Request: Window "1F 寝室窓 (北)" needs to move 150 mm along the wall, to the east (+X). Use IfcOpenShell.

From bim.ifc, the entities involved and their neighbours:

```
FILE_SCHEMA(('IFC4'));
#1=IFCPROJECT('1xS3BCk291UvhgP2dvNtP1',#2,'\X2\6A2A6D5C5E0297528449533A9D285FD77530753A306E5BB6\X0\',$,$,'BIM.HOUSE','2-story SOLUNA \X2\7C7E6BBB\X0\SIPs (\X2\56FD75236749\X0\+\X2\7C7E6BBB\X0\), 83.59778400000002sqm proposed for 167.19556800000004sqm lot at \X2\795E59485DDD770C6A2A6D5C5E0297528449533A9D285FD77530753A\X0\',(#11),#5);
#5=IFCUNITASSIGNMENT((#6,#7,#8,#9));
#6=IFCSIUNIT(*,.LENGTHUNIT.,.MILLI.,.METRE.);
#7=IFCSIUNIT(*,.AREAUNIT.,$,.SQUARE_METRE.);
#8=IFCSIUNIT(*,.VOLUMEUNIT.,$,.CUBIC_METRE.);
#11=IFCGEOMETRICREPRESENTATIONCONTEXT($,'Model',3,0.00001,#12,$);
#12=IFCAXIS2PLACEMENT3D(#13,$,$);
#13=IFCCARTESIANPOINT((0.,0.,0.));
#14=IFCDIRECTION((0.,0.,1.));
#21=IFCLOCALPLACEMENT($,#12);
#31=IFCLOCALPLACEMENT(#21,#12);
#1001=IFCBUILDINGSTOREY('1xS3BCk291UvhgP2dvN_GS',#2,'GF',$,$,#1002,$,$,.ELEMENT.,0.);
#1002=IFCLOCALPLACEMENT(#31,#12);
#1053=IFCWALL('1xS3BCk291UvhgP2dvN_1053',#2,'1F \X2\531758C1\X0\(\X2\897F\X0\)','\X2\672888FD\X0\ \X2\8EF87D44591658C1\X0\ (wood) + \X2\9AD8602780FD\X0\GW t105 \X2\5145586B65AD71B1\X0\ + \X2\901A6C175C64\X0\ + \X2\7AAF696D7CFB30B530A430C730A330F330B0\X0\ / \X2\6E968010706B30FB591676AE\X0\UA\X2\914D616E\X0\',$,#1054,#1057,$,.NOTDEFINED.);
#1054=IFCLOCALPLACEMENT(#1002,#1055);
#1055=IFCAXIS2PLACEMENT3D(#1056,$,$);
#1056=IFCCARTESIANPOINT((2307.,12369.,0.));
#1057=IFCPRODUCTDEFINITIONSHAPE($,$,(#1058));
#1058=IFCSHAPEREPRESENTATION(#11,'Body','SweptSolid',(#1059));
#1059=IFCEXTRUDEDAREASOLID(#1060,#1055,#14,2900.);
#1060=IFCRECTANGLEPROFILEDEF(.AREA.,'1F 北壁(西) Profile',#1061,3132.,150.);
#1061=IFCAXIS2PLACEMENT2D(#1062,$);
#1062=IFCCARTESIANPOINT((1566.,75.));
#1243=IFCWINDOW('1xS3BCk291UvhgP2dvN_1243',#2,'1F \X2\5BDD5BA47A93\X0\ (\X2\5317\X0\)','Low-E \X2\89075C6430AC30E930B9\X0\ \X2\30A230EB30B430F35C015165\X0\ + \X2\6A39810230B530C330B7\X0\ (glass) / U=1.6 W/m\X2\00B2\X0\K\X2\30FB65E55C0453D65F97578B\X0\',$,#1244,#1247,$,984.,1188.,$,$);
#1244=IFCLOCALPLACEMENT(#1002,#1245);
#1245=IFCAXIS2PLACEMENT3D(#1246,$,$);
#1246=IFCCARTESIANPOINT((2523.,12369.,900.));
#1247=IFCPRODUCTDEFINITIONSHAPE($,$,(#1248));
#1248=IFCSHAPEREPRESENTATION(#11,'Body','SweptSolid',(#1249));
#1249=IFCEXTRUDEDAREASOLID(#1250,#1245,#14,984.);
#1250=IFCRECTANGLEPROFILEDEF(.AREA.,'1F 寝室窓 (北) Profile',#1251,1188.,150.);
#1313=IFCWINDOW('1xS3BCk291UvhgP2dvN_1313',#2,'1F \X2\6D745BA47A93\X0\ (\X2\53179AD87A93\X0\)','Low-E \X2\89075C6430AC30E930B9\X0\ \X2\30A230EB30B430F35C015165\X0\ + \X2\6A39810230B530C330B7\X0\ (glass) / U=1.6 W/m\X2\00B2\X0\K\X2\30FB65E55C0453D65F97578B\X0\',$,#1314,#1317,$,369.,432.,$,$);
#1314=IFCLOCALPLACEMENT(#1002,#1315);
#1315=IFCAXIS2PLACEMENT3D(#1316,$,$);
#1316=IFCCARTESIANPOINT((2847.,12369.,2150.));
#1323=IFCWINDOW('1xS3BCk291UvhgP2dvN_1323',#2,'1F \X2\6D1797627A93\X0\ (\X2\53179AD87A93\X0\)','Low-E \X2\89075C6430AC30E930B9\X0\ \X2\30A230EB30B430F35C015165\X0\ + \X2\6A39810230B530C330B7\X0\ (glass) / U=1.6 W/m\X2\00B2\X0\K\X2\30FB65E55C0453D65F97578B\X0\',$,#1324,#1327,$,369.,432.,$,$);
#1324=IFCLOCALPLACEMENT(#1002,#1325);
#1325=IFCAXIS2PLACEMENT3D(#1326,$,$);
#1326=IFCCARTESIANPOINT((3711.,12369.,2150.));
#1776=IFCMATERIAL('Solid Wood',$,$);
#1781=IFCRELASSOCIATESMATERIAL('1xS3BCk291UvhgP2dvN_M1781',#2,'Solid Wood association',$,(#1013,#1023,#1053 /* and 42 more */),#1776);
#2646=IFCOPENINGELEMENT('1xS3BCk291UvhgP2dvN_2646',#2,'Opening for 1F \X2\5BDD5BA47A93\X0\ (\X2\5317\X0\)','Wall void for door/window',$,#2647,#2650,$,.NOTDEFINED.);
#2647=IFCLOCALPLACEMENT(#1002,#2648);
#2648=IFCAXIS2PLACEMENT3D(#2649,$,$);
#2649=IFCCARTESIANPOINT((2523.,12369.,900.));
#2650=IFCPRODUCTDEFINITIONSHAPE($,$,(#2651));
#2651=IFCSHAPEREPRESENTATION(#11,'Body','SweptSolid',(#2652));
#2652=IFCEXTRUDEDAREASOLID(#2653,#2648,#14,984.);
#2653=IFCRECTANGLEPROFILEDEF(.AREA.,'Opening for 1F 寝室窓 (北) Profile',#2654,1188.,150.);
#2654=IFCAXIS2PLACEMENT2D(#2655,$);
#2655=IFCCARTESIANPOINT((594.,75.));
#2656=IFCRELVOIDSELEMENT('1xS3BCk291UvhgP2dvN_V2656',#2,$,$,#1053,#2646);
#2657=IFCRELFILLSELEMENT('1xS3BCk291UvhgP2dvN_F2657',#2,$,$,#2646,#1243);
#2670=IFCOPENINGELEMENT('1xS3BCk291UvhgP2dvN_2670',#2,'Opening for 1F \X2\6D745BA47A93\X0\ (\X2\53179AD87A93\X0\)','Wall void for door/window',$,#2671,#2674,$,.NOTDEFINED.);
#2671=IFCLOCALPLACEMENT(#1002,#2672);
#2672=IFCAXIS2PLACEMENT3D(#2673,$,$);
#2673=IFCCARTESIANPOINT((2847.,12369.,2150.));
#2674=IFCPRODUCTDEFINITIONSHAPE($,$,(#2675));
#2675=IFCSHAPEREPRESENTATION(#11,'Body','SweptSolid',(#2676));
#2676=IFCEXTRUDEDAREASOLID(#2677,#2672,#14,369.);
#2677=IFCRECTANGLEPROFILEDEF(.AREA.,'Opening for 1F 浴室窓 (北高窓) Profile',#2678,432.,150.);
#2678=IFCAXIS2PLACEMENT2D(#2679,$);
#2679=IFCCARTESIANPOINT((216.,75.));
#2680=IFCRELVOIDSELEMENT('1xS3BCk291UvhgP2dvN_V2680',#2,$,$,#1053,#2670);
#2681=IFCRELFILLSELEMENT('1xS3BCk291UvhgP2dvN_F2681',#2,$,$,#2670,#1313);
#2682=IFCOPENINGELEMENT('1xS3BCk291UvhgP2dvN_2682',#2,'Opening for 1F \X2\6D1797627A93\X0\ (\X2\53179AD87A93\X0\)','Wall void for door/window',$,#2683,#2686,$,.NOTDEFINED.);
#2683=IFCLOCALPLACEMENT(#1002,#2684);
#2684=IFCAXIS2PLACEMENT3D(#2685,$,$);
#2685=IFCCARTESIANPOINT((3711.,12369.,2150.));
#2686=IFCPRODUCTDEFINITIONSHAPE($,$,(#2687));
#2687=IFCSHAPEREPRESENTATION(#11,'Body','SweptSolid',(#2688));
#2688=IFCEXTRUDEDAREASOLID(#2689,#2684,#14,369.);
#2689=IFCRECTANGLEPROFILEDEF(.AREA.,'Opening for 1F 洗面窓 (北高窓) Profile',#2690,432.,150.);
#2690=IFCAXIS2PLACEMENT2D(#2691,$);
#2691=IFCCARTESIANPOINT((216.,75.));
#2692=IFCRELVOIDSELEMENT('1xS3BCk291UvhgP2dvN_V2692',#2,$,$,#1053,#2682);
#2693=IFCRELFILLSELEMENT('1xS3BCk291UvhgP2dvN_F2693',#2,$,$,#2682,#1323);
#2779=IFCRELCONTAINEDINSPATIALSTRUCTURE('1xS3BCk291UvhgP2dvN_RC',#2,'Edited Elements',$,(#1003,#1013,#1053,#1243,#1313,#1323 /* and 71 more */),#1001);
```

```python
import ifcopenshell
import ifcopenshell.api.geometry
import ifcopenshell.util.placement

model = ifcopenshell.open("bim.ifc")

window = model.by_guid("1xS3BCk291UvhgP2dvN_1243")
opening = window.FillsVoids[0].RelatingOpeningElement
wall = opening.VoidsElements[0].RelatingBuildingElement

wall_matrix = ifcopenshell.util.placement.get_local_placement(wall.ObjectPlacement)
shift = wall_matrix[:3, 0] * 150.0
before = ifcopenshell.util.placement.get_local_placement(window.ObjectPlacement)[:3, 3].copy()

# The window is not placed relative to its opening, so move both.
for product in (opening, window):
    matrix = ifcopenshell.util.placement.get_local_placement(product.ObjectPlacement)
    matrix[:3, 3] += shift
    ifcopenshell.api.geometry.edit_object_placement(model, product=product, matrix=matrix, is_si=False)

after = ifcopenshell.util.placement.get_local_placement(window.ObjectPlacement)[:3, 3]
print("window moved by", (after - before).round(3) + 0.0)

model.write("bim_v2.ifc")
```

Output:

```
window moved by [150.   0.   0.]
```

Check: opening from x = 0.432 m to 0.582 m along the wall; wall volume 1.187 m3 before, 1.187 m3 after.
